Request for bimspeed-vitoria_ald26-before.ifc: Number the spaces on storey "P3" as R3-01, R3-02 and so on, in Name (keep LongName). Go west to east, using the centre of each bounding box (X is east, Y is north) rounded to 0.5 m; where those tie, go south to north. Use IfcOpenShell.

First a look at what the model holds.

```python
import ifcopenshell
import ifcopenshell.util.element
import ifcopenshell.util.placement

model = ifcopenshell.open("bimspeed-vitoria_ald26-before.ifc")
print(model.schema)
storey = next(s for s in model.by_type("IfcBuildingStorey") if s.Name == "P3")
spaces = [e for e in ifcopenshell.util.element.get_decomposition(storey) if e.is_a("IfcSpace")]
for e in sorted(spaces, key=lambda e: e.id()):
    origin = ifcopenshell.util.placement.get_local_placement(e.ObjectPlacement)[:3, 3]
    print(e.id(), e.Name, e.LongName, origin.round(2) + 0.0, sep=" | ")
```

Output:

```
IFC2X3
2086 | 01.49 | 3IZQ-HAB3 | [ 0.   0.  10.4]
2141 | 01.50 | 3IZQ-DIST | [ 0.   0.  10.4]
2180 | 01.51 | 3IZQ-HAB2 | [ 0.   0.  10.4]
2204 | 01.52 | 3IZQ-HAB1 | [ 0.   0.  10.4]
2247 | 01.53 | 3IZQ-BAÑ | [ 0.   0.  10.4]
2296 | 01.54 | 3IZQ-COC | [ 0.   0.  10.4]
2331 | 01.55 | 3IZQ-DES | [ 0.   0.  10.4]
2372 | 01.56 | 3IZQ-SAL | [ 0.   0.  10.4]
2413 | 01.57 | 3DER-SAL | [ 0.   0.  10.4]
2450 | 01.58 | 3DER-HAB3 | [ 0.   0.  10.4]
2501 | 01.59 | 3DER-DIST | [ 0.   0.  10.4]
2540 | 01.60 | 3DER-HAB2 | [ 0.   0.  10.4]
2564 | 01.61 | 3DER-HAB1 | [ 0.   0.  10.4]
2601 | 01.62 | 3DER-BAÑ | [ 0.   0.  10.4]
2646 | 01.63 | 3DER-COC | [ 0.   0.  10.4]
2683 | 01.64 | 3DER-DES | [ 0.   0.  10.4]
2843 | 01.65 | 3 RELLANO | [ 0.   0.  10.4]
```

```python
import ifcopenshell
import ifcopenshell.geom
import ifcopenshell.util.element
import ifcopenshell.util.shape

model = ifcopenshell.open("bimspeed-vitoria_ald26-before.ifc")
settings = ifcopenshell.geom.settings()
settings.set("use-world-coords", True)


def centre(element):
    shape = ifcopenshell.geom.create_shape(settings, element)
    return ifcopenshell.util.shape.get_bbox_centroid(shape.geometry)


storey = next(s for s in model.by_type("IfcBuildingStorey") if s.Name == "P3")
spaces = [e for e in ifcopenshell.util.element.get_decomposition(storey) if e.is_a("IfcSpace")]

# Insertion points can sit at a corner or the storey origin, so sort by the geometry (in metres).
centres = {e: centre(e) for e in spaces}
spaces.sort(key=lambda e: (round(centres[e][0] / 0.5), centres[e][1]))

for i, e in enumerate(spaces, start=1):
    number = f"R3-{i:02d}"
    e.Name = number
    print(e.id(), number)

model.write("bimspeed-vitoria_ald26-before_edited.ifc")
```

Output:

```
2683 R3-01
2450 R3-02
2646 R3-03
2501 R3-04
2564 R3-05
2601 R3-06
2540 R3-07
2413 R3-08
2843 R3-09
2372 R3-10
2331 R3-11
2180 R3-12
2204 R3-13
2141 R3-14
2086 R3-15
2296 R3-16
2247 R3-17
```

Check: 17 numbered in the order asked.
